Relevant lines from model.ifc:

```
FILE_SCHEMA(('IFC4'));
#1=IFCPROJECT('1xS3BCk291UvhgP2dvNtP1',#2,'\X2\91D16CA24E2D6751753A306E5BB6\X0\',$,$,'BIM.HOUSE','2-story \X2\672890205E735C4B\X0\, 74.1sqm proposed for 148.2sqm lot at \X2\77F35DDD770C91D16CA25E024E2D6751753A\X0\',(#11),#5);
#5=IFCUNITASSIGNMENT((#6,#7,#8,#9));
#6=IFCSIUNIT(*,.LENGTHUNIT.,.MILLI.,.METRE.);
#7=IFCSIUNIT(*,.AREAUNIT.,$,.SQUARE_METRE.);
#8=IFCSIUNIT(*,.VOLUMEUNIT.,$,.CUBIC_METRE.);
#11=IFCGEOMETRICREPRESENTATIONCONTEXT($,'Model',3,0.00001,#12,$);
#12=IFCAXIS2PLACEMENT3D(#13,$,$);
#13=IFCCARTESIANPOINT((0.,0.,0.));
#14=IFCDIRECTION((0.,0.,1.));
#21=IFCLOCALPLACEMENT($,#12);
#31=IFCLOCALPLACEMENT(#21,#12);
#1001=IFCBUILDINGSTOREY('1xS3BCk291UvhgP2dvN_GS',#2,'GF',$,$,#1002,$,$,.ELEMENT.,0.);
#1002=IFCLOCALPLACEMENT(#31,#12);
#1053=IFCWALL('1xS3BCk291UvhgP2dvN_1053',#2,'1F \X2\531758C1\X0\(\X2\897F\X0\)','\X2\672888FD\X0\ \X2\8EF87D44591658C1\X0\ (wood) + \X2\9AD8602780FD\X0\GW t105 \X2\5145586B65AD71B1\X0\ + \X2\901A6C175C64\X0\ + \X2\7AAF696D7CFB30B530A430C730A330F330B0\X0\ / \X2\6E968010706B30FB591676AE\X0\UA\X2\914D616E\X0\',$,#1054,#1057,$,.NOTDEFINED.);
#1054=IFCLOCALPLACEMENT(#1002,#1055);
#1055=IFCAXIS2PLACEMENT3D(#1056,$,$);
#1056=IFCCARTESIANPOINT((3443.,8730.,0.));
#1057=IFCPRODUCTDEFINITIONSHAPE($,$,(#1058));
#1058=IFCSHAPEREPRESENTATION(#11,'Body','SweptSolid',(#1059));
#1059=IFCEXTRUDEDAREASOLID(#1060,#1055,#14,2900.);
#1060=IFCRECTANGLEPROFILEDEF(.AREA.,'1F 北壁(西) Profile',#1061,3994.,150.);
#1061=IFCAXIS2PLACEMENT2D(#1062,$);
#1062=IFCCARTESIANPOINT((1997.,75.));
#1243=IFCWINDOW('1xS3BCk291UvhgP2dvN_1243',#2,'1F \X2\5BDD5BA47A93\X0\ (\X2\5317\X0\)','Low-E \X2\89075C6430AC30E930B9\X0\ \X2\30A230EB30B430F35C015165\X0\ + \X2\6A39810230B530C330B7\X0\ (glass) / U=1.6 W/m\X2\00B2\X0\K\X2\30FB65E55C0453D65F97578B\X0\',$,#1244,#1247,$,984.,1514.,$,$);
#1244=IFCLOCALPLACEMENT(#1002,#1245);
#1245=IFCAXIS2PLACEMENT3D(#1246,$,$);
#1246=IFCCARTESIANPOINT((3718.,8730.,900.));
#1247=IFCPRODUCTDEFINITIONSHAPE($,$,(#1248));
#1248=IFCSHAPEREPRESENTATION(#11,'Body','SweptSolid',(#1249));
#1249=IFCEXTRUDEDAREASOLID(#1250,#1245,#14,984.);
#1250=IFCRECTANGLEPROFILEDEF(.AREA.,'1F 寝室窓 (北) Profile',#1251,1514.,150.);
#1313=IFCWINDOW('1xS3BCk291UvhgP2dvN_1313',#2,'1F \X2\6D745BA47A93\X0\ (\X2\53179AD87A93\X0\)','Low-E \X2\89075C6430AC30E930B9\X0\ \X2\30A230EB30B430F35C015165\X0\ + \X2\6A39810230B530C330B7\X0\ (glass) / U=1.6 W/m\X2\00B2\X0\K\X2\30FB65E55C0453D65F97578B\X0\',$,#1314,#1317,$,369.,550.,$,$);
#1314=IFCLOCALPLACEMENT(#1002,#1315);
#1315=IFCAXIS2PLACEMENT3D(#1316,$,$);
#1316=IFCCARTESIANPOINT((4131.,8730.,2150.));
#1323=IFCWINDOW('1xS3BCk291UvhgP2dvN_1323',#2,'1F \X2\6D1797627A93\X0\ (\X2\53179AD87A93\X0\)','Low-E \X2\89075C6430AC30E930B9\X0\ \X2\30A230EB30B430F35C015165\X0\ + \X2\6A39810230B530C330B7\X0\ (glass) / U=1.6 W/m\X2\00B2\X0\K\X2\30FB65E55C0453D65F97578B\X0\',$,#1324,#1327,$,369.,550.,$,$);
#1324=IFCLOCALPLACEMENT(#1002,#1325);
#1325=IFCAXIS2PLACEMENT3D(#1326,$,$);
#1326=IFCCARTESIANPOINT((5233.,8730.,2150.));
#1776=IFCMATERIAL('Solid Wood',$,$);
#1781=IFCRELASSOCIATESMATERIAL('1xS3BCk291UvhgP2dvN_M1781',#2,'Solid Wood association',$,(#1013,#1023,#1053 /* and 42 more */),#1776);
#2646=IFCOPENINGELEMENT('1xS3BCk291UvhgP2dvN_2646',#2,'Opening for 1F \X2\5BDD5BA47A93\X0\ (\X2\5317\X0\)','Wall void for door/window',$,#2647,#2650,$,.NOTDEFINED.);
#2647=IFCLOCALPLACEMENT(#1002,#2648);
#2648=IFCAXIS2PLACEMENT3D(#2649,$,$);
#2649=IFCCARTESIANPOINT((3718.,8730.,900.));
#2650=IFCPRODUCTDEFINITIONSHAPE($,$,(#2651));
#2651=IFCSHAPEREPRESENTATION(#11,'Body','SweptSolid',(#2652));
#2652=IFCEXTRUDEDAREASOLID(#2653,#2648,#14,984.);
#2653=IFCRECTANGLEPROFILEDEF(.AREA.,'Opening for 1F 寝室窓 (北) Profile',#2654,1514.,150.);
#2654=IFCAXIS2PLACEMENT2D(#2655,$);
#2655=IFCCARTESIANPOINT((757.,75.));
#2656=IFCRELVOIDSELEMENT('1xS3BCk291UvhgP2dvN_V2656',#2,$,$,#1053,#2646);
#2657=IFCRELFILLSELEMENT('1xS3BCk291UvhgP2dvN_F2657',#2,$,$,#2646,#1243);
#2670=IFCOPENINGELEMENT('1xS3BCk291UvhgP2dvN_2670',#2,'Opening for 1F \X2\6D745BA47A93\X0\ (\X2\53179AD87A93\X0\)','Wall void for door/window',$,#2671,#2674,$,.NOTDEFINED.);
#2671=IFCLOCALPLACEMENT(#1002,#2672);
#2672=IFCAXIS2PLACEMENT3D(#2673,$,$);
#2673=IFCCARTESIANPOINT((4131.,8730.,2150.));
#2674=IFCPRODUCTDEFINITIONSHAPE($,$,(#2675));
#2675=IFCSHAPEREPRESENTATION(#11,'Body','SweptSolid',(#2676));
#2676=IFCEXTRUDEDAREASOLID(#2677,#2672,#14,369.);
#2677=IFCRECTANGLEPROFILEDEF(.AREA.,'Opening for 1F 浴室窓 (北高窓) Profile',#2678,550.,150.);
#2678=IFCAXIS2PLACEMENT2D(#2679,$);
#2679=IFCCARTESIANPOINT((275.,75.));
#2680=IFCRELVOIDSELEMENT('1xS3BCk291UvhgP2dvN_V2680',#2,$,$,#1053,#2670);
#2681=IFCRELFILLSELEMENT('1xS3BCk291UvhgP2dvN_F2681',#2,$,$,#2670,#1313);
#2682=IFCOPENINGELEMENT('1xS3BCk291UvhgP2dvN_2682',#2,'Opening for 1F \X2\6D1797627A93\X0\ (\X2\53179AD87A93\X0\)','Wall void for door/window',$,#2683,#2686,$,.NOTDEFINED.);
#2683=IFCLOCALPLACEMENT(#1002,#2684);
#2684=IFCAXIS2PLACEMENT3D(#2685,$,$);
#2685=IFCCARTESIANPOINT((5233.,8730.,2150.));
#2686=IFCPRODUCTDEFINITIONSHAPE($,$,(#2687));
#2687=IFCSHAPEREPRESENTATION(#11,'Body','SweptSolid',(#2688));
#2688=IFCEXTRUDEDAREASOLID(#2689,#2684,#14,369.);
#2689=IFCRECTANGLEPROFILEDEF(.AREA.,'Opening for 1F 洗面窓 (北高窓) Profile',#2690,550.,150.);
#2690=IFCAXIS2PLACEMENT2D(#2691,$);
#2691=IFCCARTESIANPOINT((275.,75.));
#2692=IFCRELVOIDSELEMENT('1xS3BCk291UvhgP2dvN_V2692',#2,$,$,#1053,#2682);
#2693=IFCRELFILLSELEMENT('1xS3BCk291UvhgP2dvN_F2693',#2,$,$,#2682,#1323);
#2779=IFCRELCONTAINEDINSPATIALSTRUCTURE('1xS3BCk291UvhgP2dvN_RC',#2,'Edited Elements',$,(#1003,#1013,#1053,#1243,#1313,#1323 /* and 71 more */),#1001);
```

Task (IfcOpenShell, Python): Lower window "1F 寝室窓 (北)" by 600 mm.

```python
import numpy as np
import ifcopenshell
import ifcopenshell.api.geometry
import ifcopenshell.util.placement
import ifcopenshell.util.unit

model = ifcopenshell.open("model.ifc")
unit_scale = ifcopenshell.util.unit.calculate_unit_scale(model)

window = model.by_id(1243)
opening = window.FillsVoids[0].RelatingOpeningElement
dz = -600.0

shift = np.array([0.0, 0.0, dz])
# The window is not placed relative to its opening, so move both.
for product in (opening, window):
    matrix = ifcopenshell.util.placement.get_local_placement(product.ObjectPlacement)
    matrix[:3, 3] += shift
    ifcopenshell.api.geometry.edit_object_placement(model, product=product, matrix=matrix, is_si=False)

print(f"moved by {dz * unit_scale:+.3f} m")

model.write("model_edited.ifc")
```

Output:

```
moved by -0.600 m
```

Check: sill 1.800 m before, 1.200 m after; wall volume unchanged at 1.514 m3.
